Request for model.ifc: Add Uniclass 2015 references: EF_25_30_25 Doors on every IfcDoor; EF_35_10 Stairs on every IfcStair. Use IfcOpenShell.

First a look at what the model holds.

```python
import ifcopenshell

model = ifcopenshell.open("model.ifc")
print(model.schema)
print("classifications:", [c.Name for c in model.by_type("IfcClassification")])
for ifc_class in ("IfcDoor", "IfcRoof", "IfcStair", "IfcWall", "IfcWindow"):
    print(ifc_class, len(model.by_type(ifc_class)))
```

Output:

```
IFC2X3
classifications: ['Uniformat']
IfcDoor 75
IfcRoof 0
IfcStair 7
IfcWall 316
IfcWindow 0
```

```python
import ifcopenshell
import ifcopenshell.api.classification

model = ifcopenshell.open("model.ifc")

# IFC2X3 requires Source and Edition and has no link from the project to the system.
system = model.create_entity("IfcClassification", Source="NBS", Edition="2015", Name="Uniclass 2015")

codes = {
    "IfcDoor": ("EF_25_30_25", "Doors"),
    "IfcStair": ("EF_35_10", "Stairs"),
}
for ifc_class, (code, name) in codes.items():
    products = model.by_type(ifc_class)
    ifcopenshell.api.classification.add_reference(
        model, products=products, classification=system, identification=code, name=name
    )
    print(code, len(products))

model.write("model_updated.ifc")
```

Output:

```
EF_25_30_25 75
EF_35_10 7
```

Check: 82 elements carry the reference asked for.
